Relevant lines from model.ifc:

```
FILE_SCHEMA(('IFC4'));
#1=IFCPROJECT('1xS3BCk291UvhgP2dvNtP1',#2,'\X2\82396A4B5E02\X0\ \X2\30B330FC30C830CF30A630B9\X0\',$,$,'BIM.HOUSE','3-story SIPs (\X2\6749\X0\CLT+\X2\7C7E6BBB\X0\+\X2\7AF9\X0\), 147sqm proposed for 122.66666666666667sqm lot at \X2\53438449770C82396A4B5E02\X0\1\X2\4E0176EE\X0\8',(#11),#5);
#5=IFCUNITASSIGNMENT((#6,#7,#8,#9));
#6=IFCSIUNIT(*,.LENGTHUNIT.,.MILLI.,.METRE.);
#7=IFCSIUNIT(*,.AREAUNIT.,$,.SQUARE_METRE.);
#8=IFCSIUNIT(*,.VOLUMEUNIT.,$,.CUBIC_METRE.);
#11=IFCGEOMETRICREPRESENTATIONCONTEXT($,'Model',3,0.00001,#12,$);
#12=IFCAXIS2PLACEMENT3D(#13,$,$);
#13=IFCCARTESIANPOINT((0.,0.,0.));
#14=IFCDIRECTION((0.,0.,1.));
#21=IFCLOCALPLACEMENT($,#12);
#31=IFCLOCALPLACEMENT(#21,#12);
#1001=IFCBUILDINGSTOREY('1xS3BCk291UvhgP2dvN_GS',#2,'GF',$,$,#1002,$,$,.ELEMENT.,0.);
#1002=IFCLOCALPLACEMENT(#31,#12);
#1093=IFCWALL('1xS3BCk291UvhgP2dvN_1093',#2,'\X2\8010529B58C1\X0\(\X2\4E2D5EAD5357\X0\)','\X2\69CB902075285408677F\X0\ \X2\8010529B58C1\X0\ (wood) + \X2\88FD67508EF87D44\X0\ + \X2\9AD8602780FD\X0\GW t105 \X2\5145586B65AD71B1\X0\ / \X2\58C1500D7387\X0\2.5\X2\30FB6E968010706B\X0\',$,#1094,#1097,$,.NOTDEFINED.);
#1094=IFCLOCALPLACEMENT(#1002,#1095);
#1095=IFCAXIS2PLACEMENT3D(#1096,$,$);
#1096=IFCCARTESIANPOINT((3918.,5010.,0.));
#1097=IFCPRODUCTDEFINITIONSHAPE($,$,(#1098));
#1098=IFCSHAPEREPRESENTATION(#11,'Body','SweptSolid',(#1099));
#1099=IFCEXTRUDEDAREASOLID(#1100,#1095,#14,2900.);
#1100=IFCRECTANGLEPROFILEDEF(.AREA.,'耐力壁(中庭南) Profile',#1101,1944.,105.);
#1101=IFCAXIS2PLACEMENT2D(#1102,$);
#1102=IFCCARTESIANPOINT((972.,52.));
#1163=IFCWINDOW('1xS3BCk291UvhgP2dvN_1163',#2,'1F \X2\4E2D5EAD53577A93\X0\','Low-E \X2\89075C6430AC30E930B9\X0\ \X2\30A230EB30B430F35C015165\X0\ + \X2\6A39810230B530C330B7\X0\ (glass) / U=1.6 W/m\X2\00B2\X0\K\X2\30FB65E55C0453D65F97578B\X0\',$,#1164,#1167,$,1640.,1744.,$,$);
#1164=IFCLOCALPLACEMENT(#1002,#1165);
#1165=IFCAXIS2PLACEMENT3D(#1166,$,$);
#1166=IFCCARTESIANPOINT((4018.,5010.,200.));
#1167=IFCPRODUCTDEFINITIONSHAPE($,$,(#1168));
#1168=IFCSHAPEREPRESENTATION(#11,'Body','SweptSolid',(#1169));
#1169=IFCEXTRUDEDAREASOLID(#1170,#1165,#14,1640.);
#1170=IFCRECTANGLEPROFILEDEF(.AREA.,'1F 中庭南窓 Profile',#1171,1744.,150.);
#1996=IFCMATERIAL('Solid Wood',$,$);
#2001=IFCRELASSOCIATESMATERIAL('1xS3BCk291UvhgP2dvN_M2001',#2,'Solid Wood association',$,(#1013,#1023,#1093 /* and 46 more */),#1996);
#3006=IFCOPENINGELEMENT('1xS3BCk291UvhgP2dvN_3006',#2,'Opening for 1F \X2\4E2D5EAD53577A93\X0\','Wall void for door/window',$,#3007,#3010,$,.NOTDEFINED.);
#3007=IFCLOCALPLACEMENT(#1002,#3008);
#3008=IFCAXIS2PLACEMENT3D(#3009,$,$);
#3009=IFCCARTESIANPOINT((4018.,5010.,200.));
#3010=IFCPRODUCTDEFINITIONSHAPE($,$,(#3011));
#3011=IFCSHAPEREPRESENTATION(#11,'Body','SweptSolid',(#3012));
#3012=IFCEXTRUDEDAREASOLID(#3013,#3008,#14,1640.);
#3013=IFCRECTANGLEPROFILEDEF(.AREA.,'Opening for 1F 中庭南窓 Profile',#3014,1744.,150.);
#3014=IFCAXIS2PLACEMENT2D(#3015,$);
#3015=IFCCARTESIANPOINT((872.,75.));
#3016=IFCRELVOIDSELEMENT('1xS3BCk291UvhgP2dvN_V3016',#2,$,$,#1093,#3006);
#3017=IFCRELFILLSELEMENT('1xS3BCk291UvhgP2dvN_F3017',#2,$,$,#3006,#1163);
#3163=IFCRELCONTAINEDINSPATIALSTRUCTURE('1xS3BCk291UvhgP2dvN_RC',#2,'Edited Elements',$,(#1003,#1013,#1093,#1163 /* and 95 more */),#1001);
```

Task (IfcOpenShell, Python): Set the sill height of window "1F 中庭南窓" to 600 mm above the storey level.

```python
import numpy as np
import ifcopenshell
import ifcopenshell.api.geometry
import ifcopenshell.geom
import ifcopenshell.util.element
import ifcopenshell.util.placement
import ifcopenshell.util.shape
import ifcopenshell.util.unit

model = ifcopenshell.open("model.ifc")
unit_scale = ifcopenshell.util.unit.calculate_unit_scale(model)

window = model.by_id(1163)
opening = window.FillsVoids[0].RelatingOpeningElement
storey = ifcopenshell.util.element.get_container(window, ifc_class="IfcBuildingStorey")
level = ifcopenshell.util.placement.get_local_placement(storey.ObjectPlacement)[2, 3]

# The opening's origin need not be at the sill, so measure its lowest point.
shape = ifcopenshell.geom.create_shape(ifcopenshell.geom.settings(), opening)
bottom = ifcopenshell.util.shape.get_shape_bottom_elevation(shape, shape.geometry) / unit_scale
dz = level + 0.6 / unit_scale - bottom

shift = np.array([0.0, 0.0, dz])
# The window is not placed relative to its opening, so move both.
for product in (opening, window):
    matrix = ifcopenshell.util.placement.get_local_placement(product.ObjectPlacement)
    matrix[:3, 3] += shift
    ifcopenshell.api.geometry.edit_object_placement(model, product=product, matrix=matrix, is_si=False)

print(f"moved by {dz * unit_scale:+.3f} m")

model.write("model_rev.ifc")
```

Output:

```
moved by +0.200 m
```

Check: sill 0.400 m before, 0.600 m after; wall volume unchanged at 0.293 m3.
